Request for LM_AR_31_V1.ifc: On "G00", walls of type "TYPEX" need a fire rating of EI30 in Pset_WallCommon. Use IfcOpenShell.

First a look at what the model holds.

```python
import ifcopenshell
import ifcopenshell.util.element

model = ifcopenshell.open("LM_AR_31_V1.ifc")
print(model.schema)
storey = next(s for s in model.by_type("IfcBuildingStorey") if s.Name == "G00")
walls = [e for e in ifcopenshell.util.element.get_decomposition(storey) if e.is_a("IfcWall")]
seen = {}
for e in walls:
    element_type = ifcopenshell.util.element.get_type(e)
    key = (element_type.Name if element_type != e and element_type else None, ifcopenshell.util.element.get_pset(e, "Pset_WallCommon", "FireRating"))
    seen[key] = seen.get(key, 0) + 1
for (name, value), count in sorted(seen.items(), key=str):
    print(count, "x", name, "|", value)
```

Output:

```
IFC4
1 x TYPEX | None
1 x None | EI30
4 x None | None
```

```python
import ifcopenshell
import ifcopenshell.api.pset
import ifcopenshell.util.element

model = ifcopenshell.open("LM_AR_31_V1.ifc")

storey = next(s for s in model.by_type("IfcBuildingStorey") if s.Name == "G00")
walls = [e for e in ifcopenshell.util.element.get_decomposition(storey) if e.is_a("IfcWall")]

count = 0
for e in walls:
    element_type = ifcopenshell.util.element.get_type(e)
    if element_type in (None, e) or element_type.Name != "TYPEX":
        continue
    # add_pset returns the element's existing set when there is one.
    pset = ifcopenshell.api.pset.add_pset(model, product=e, name="Pset_WallCommon")
    ifcopenshell.api.pset.edit_pset(model, pset=pset, properties={"FireRating": "EI30"})
    count += 1

print(count, "walls updated")

model.write("LM_AR_31_V1_updated.ifc")
```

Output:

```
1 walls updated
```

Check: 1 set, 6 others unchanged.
